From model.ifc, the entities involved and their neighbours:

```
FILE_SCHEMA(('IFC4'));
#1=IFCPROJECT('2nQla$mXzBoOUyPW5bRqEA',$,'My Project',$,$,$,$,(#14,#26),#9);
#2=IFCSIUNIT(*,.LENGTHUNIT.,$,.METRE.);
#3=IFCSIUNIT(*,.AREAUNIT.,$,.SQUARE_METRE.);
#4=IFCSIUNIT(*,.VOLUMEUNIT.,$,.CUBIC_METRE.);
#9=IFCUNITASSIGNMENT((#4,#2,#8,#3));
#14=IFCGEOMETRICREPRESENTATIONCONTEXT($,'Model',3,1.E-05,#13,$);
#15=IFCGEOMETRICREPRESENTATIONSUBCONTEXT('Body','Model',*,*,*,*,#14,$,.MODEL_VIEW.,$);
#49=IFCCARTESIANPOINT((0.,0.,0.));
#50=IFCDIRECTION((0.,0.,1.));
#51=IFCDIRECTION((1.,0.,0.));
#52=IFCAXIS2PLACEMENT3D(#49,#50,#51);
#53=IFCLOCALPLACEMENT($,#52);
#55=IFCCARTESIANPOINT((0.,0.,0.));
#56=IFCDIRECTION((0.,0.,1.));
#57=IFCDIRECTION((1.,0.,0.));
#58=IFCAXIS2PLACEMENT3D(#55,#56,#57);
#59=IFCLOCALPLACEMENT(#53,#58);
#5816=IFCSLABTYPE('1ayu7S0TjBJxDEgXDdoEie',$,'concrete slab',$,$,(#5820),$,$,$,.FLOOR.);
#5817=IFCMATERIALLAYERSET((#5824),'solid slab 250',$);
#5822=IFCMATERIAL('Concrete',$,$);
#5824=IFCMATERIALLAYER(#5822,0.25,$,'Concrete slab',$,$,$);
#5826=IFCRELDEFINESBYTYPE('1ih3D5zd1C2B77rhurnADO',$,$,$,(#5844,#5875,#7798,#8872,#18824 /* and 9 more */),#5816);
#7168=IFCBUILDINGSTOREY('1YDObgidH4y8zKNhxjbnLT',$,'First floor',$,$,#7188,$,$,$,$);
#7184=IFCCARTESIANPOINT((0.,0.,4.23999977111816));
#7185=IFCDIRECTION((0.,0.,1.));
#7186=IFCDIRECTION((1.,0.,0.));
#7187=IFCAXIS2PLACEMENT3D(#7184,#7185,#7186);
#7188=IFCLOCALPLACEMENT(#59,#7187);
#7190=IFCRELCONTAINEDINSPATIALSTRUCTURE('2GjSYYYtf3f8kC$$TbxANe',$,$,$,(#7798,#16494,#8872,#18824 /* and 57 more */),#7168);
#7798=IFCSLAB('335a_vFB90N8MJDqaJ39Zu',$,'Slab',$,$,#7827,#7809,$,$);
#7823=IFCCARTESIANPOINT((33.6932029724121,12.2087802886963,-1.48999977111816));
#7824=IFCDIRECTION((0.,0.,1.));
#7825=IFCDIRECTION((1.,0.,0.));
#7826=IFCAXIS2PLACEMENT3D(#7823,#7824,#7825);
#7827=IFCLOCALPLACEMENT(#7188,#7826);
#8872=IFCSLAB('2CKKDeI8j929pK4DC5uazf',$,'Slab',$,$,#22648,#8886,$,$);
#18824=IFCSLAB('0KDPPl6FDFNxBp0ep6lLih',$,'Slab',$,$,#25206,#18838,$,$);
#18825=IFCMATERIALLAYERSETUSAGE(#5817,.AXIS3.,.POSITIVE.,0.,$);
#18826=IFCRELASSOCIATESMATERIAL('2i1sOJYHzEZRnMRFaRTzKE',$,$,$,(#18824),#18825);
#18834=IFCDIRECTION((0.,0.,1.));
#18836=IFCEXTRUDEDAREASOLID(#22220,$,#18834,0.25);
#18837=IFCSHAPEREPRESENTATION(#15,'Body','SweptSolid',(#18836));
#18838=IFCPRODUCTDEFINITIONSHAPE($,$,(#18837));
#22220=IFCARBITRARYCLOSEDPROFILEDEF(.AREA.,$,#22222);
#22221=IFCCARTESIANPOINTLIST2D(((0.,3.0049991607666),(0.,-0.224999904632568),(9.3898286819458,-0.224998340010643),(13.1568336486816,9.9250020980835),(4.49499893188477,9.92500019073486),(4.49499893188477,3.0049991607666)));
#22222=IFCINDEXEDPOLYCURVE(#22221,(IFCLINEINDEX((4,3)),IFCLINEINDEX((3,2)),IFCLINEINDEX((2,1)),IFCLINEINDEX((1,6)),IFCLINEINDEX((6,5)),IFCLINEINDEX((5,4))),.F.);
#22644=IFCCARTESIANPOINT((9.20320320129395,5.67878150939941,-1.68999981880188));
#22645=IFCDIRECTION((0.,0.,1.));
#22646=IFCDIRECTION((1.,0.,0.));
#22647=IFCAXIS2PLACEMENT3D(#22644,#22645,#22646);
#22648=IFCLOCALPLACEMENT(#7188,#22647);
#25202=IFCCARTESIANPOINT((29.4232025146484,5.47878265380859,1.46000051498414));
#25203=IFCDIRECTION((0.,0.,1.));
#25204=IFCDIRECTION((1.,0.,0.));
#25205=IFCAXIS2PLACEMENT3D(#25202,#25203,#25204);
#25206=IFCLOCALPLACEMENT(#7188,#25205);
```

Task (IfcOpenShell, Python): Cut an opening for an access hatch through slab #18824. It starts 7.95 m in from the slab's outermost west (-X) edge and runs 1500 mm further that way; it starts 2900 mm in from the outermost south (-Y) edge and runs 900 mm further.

```python
import numpy as np
import ifcopenshell
import ifcopenshell.api.feature
import ifcopenshell.api.geometry
import ifcopenshell.api.root
import ifcopenshell.geom
import ifcopenshell.util.placement
import ifcopenshell.util.representation
import ifcopenshell.util.shape
import ifcopenshell.util.unit

model = ifcopenshell.open("model.ifc")
unit_scale = ifcopenshell.util.unit.calculate_unit_scale(model)
settings = ifcopenshell.geom.settings()


def volume(element):
    """Net volume in cubic metres, openings subtracted."""
    shape = ifcopenshell.geom.create_shape(settings, element)
    return ifcopenshell.util.shape.get_volume(shape.geometry)


slab = model.by_guid("0KDPPl6FDFNxBp0ep6lLih")
before = volume(slab)

# Extent in the slab's own axes, in metres. The edges named are its -X and -Y sides.
slab_shape = ifcopenshell.geom.create_shape(settings, slab)
vertices = ifcopenshell.util.shape.get_vertices(slab_shape.geometry)
x_min, y_min, bottom = vertices.min(axis=0)
top = vertices[:, 2].max()

opening = ifcopenshell.api.root.create_entity(model, ifc_class="IfcOpeningElement", name="Access hatch opening", predefined_type="OPENING")
context = ifcopenshell.util.representation.get_context(model, "Model", "Body", "MODEL_VIEW")
width, depth = 1.5, 0.9
outline = [(0.0, 0.0), (width, 0.0), (width, depth), (0.0, depth), (0.0, 0.0)]
# Overshoot both faces by 50 mm so the cut is clean.
shape = ifcopenshell.api.geometry.add_slab_representation(
    model, context=context, depth=top - bottom + 0.1, polyline=outline
)
ifcopenshell.api.geometry.assign_representation(model, product=opening, representation=shape)

matrix = ifcopenshell.util.placement.get_local_placement(slab.ObjectPlacement)
matrix[:, 3] = matrix @ np.append(np.array([x_min + 7.95, y_min + 2.9, bottom - 0.05]) / unit_scale, 1.0)
ifcopenshell.api.geometry.edit_object_placement(model, product=opening, matrix=matrix, is_si=False)
ifcopenshell.api.feature.add_feature(model, feature=opening, element=slab)

after = volume(slab)

print(f"slab volume {before:.3f} -> {after:.3f} m3")

model.write("model_v2.ifc")
```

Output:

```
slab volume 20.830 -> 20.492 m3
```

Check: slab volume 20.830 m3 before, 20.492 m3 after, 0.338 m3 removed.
